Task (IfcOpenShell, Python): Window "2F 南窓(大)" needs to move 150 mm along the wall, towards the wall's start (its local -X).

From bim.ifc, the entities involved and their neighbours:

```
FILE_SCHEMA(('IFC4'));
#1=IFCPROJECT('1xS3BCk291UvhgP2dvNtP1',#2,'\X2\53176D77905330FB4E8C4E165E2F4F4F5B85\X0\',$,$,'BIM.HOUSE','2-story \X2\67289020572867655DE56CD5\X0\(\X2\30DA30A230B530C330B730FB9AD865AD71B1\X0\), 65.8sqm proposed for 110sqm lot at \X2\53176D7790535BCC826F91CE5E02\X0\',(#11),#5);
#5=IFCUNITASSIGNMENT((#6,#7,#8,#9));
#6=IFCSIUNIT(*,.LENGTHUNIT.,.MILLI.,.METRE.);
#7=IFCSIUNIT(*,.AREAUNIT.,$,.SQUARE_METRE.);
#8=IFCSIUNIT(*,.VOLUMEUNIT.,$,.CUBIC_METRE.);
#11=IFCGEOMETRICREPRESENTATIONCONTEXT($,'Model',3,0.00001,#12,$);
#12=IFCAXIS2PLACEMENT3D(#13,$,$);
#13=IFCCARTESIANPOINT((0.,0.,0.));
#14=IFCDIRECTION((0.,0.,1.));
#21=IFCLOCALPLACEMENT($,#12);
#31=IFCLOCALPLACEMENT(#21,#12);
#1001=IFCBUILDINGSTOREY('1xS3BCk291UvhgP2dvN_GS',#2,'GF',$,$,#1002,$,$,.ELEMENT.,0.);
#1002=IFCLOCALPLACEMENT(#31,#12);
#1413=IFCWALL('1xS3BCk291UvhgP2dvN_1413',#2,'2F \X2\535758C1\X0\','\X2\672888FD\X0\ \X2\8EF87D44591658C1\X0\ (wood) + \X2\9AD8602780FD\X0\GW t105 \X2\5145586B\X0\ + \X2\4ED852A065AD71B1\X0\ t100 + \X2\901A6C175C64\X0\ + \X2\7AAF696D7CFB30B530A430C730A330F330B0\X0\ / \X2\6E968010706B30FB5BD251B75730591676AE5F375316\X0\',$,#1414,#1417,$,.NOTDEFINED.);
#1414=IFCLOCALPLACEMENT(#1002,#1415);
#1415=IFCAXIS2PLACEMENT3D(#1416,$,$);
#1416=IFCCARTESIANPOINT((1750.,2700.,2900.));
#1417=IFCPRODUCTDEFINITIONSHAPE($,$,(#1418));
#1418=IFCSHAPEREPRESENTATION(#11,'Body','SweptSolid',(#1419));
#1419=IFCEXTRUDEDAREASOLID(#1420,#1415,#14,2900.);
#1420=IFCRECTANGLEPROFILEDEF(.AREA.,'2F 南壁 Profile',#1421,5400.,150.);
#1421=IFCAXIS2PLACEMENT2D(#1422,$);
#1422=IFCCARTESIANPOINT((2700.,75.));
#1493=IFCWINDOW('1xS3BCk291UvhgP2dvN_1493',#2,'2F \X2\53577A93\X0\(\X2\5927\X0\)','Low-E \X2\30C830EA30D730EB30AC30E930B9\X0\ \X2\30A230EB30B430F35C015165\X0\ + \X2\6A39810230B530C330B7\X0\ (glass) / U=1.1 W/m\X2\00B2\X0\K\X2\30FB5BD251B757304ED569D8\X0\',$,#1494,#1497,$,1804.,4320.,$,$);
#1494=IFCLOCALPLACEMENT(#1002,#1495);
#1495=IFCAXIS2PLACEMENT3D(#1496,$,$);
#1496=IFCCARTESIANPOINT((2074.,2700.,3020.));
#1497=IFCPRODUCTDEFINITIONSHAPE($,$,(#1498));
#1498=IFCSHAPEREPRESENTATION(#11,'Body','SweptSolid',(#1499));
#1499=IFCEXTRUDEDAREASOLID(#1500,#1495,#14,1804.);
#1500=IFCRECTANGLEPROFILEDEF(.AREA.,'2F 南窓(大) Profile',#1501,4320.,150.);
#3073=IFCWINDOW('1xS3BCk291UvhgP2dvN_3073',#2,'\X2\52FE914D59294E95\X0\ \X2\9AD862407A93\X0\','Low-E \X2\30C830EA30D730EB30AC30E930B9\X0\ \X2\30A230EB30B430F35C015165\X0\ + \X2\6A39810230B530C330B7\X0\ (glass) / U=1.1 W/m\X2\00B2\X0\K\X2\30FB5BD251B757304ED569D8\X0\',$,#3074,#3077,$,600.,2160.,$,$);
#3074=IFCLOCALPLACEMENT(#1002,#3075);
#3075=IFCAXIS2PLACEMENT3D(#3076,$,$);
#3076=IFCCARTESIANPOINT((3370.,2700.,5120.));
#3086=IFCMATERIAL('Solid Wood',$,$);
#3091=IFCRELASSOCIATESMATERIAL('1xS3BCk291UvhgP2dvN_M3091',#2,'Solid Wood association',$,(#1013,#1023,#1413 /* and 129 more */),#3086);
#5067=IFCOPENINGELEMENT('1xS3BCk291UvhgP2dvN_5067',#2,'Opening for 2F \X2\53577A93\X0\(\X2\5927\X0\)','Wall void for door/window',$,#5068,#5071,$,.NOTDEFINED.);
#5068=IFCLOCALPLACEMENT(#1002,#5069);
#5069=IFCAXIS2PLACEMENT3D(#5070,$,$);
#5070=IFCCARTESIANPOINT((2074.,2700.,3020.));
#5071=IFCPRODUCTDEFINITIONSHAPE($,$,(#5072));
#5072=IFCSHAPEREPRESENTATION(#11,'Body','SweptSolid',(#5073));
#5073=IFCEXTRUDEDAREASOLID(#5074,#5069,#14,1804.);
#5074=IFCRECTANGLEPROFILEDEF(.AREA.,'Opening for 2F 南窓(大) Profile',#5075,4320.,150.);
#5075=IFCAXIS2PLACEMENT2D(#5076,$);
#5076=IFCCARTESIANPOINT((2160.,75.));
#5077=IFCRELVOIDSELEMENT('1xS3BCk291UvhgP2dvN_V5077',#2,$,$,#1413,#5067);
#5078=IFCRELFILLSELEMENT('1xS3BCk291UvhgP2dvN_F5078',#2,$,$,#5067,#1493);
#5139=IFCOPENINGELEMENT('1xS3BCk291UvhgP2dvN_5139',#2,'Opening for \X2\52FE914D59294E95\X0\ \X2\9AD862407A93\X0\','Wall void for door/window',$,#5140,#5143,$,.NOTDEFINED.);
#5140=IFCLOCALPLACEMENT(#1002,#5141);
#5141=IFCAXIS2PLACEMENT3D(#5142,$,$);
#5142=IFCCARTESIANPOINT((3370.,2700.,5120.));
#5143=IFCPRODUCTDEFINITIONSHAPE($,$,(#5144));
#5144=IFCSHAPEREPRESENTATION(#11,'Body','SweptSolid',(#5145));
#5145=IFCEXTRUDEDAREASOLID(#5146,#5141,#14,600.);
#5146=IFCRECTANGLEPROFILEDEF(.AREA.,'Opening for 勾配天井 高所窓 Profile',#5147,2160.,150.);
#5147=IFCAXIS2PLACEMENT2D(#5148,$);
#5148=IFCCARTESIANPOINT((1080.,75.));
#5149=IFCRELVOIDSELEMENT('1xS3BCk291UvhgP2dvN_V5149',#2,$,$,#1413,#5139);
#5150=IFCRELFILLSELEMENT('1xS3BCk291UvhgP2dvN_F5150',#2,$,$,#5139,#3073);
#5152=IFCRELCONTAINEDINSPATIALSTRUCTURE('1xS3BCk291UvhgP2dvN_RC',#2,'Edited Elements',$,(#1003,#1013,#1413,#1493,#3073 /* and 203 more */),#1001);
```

```python
import ifcopenshell
import ifcopenshell.api.geometry
import ifcopenshell.util.placement

model = ifcopenshell.open("bim.ifc")

window = model.by_id(1493)
opening = window.FillsVoids[0].RelatingOpeningElement
wall = opening.VoidsElements[0].RelatingBuildingElement

wall_matrix = ifcopenshell.util.placement.get_local_placement(wall.ObjectPlacement)
shift = wall_matrix[:3, 0] * -150.0
before = ifcopenshell.util.placement.get_local_placement(window.ObjectPlacement)[:3, 3].copy()

# The window is not placed relative to its opening, so move both.
for product in (opening, window):
    matrix = ifcopenshell.util.placement.get_local_placement(product.ObjectPlacement)
    matrix[:3, 3] += shift
    ifcopenshell.api.geometry.edit_object_placement(model, product=product, matrix=matrix, is_si=False)

after = ifcopenshell.util.placement.get_local_placement(window.ObjectPlacement)[:3, 3]
print("window moved by", (after - before).round(3) + 0.0)

model.write("bim_updated.ifc")
```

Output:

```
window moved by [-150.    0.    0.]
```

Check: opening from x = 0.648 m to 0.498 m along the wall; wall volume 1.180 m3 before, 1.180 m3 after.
